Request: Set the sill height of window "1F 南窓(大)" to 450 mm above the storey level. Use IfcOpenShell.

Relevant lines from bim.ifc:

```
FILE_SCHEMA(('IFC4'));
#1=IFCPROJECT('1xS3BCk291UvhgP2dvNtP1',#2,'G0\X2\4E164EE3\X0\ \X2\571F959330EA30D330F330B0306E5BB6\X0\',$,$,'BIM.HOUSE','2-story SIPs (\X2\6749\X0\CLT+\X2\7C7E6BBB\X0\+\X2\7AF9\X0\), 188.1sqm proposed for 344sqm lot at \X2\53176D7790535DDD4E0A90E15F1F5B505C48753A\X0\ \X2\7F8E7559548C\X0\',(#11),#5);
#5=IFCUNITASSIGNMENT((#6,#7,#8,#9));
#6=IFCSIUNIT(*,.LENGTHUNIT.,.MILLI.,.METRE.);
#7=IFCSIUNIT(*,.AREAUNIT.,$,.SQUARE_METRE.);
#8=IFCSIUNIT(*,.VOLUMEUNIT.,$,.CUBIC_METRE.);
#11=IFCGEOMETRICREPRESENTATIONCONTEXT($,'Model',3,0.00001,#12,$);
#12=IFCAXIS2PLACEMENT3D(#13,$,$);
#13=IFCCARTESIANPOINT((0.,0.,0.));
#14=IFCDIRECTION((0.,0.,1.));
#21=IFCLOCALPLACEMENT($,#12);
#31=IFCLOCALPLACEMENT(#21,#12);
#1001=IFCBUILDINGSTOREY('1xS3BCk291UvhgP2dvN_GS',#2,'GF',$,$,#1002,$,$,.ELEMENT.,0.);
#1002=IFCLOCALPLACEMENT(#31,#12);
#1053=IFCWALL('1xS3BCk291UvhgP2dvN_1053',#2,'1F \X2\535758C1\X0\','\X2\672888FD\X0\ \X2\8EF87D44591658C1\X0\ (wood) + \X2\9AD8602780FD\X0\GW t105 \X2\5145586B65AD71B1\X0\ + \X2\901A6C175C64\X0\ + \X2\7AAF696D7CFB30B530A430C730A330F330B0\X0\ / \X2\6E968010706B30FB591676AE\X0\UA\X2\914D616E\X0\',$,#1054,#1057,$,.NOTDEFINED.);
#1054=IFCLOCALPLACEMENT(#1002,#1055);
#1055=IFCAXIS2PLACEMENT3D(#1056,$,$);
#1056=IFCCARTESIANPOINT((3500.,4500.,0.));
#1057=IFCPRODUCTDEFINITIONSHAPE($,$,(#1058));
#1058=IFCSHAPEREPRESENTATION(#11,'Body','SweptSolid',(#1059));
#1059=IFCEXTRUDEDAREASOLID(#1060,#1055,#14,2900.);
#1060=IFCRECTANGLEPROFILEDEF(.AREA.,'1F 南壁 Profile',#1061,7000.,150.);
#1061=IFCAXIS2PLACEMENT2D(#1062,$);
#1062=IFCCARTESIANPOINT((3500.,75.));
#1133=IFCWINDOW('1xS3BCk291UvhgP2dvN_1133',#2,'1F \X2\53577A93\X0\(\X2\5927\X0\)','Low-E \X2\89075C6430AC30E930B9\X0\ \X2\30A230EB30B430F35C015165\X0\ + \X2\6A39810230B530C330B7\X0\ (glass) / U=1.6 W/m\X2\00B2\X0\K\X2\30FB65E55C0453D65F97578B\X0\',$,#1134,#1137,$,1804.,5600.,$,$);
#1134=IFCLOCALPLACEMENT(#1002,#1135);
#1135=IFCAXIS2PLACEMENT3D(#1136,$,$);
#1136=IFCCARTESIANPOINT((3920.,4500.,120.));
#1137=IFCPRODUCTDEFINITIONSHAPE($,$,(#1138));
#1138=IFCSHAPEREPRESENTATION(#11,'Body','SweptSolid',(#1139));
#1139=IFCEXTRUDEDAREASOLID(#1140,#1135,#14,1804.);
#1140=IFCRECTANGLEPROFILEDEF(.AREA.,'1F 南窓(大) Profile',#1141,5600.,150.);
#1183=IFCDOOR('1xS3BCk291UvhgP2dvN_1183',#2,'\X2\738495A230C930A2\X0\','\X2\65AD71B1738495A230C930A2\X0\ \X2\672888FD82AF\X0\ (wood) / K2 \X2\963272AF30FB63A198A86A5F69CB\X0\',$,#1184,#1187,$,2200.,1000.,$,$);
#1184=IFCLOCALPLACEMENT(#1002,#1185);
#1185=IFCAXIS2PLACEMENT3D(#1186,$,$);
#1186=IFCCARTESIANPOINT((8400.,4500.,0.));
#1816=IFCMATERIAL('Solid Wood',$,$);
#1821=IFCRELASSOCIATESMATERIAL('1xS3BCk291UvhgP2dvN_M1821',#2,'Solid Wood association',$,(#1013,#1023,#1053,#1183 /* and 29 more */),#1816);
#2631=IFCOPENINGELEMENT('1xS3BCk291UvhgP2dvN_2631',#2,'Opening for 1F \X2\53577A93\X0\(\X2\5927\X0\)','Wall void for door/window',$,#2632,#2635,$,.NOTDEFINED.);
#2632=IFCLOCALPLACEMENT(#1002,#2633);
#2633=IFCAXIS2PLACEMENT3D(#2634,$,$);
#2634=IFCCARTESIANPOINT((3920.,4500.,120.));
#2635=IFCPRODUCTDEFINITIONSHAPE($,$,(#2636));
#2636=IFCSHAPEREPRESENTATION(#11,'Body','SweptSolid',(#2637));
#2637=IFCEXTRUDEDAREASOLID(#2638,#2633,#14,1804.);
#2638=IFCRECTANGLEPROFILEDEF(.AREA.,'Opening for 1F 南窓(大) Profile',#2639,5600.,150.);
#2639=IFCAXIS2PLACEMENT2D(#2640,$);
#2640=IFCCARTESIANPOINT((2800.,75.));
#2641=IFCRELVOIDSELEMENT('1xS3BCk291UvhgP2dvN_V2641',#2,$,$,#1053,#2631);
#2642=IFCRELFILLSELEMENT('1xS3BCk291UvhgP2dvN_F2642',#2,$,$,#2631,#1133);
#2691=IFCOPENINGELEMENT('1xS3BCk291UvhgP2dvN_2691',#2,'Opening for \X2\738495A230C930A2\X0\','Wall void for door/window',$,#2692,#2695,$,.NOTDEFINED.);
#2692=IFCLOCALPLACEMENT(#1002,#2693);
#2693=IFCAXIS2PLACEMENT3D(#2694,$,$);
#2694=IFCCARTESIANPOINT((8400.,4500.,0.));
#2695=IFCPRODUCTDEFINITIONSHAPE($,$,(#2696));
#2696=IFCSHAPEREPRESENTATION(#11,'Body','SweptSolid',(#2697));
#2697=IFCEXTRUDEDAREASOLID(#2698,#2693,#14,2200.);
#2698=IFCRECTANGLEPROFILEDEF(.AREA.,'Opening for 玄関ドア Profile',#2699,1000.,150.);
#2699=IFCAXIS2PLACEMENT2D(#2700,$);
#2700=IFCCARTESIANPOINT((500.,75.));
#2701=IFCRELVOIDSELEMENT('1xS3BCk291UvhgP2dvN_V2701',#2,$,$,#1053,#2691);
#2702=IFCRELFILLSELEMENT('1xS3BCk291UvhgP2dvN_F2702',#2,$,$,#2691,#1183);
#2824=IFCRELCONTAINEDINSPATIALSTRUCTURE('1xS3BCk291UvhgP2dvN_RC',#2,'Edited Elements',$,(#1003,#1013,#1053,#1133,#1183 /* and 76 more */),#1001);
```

```python
import numpy as np
import ifcopenshell
import ifcopenshell.api.geometry
import ifcopenshell.geom
import ifcopenshell.util.element
import ifcopenshell.util.placement
import ifcopenshell.util.shape
import ifcopenshell.util.unit

model = ifcopenshell.open("bim.ifc")
unit_scale = ifcopenshell.util.unit.calculate_unit_scale(model)

window = model.by_id(1133)
opening = window.FillsVoids[0].RelatingOpeningElement
storey = ifcopenshell.util.element.get_container(window, ifc_class="IfcBuildingStorey")
level = ifcopenshell.util.placement.get_local_placement(storey.ObjectPlacement)[2, 3]

# The opening's origin need not be at the sill, so measure its lowest point.
shape = ifcopenshell.geom.create_shape(ifcopenshell.geom.settings(), opening)
bottom = ifcopenshell.util.shape.get_shape_bottom_elevation(shape, shape.geometry) / unit_scale
dz = level + 0.45 / unit_scale - bottom

shift = np.array([0.0, 0.0, dz])
# The window is not placed relative to its opening, so move both.
for product in (opening, window):
    matrix = ifcopenshell.util.placement.get_local_placement(product.ObjectPlacement)
    matrix[:3, 3] += shift
    ifcopenshell.api.geometry.edit_object_placement(model, product=product, matrix=matrix, is_si=False)

print(f"moved by {dz * unit_scale:+.3f} m")

model.write("bim_edited.ifc")
```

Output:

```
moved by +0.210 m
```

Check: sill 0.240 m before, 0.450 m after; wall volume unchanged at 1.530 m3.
